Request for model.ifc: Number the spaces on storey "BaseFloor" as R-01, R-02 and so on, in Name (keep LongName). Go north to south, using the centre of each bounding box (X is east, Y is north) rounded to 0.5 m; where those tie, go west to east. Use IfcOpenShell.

First a look at what the model holds.

```python
import ifcopenshell
import ifcopenshell.util.element
import ifcopenshell.util.placement

model = ifcopenshell.open("model.ifc")
print(model.schema)
storey = next(s for s in model.by_type("IfcBuildingStorey") if s.Name == "BaseFloor")
spaces = [e for e in ifcopenshell.util.element.get_decomposition(storey) if e.is_a("IfcSpace")]
for e in sorted(spaces, key=lambda e: e.id()):
    origin = ifcopenshell.util.placement.get_local_placement(e.ObjectPlacement)[:3, 3]
    print(e.id(), e.Name, e.LongName, origin.round(2) + 0.0, sep=" | ")
```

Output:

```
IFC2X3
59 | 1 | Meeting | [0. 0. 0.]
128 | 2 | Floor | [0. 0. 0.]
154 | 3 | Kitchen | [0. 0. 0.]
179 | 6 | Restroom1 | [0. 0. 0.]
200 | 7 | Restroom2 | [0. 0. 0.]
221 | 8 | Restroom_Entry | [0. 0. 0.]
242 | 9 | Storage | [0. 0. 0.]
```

```python
import ifcopenshell
import ifcopenshell.geom
import ifcopenshell.util.element
import ifcopenshell.util.shape

model = ifcopenshell.open("model.ifc")
settings = ifcopenshell.geom.settings()
settings.set("use-world-coords", True)


def centre(element):
    shape = ifcopenshell.geom.create_shape(settings, element)
    return ifcopenshell.util.shape.get_bbox_centroid(shape.geometry)


storey = next(s for s in model.by_type("IfcBuildingStorey") if s.Name == "BaseFloor")
spaces = [e for e in ifcopenshell.util.element.get_decomposition(storey) if e.is_a("IfcSpace")]

# Insertion points can sit at a corner or the storey origin, so sort by the geometry (in metres).
centres = {e: centre(e) for e in spaces}
spaces.sort(key=lambda e: (-round(centres[e][1] / 0.5), centres[e][0]))

for i, e in enumerate(spaces, start=1):
    number = f"R-{i:02d}"
    e.Name = number
    print(e.id(), number)

model.write("model_updated.ifc")
```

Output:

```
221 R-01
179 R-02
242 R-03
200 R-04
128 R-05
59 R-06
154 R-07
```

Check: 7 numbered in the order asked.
